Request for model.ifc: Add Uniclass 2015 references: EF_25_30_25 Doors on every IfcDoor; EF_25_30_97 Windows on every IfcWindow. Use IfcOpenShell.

First a look at what the model holds.

```python
import ifcopenshell

model = ifcopenshell.open("model.ifc")
print(model.schema)
print("classifications:", [c.Name for c in model.by_type("IfcClassification")])
for ifc_class in ("IfcDoor", "IfcRoof", "IfcStair", "IfcWall", "IfcWindow"):
    print(ifc_class, len(model.by_type(ifc_class)))
```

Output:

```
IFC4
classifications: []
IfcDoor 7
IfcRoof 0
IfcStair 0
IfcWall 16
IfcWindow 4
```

```python
import ifcopenshell
import ifcopenshell.api.classification

model = ifcopenshell.open("model.ifc")

system = ifcopenshell.api.classification.add_classification(model, classification="Uniclass 2015")

codes = {
    "IfcDoor": ("EF_25_30_25", "Doors"),
    "IfcWindow": ("EF_25_30_97", "Windows"),
}
for ifc_class, (code, name) in codes.items():
    products = model.by_type(ifc_class)
    ifcopenshell.api.classification.add_reference(
        model, products=products, classification=system, identification=code, name=name
    )
    print(code, len(products))

model.write("model_v2.ifc")
```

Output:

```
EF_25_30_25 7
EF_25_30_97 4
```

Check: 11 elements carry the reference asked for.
